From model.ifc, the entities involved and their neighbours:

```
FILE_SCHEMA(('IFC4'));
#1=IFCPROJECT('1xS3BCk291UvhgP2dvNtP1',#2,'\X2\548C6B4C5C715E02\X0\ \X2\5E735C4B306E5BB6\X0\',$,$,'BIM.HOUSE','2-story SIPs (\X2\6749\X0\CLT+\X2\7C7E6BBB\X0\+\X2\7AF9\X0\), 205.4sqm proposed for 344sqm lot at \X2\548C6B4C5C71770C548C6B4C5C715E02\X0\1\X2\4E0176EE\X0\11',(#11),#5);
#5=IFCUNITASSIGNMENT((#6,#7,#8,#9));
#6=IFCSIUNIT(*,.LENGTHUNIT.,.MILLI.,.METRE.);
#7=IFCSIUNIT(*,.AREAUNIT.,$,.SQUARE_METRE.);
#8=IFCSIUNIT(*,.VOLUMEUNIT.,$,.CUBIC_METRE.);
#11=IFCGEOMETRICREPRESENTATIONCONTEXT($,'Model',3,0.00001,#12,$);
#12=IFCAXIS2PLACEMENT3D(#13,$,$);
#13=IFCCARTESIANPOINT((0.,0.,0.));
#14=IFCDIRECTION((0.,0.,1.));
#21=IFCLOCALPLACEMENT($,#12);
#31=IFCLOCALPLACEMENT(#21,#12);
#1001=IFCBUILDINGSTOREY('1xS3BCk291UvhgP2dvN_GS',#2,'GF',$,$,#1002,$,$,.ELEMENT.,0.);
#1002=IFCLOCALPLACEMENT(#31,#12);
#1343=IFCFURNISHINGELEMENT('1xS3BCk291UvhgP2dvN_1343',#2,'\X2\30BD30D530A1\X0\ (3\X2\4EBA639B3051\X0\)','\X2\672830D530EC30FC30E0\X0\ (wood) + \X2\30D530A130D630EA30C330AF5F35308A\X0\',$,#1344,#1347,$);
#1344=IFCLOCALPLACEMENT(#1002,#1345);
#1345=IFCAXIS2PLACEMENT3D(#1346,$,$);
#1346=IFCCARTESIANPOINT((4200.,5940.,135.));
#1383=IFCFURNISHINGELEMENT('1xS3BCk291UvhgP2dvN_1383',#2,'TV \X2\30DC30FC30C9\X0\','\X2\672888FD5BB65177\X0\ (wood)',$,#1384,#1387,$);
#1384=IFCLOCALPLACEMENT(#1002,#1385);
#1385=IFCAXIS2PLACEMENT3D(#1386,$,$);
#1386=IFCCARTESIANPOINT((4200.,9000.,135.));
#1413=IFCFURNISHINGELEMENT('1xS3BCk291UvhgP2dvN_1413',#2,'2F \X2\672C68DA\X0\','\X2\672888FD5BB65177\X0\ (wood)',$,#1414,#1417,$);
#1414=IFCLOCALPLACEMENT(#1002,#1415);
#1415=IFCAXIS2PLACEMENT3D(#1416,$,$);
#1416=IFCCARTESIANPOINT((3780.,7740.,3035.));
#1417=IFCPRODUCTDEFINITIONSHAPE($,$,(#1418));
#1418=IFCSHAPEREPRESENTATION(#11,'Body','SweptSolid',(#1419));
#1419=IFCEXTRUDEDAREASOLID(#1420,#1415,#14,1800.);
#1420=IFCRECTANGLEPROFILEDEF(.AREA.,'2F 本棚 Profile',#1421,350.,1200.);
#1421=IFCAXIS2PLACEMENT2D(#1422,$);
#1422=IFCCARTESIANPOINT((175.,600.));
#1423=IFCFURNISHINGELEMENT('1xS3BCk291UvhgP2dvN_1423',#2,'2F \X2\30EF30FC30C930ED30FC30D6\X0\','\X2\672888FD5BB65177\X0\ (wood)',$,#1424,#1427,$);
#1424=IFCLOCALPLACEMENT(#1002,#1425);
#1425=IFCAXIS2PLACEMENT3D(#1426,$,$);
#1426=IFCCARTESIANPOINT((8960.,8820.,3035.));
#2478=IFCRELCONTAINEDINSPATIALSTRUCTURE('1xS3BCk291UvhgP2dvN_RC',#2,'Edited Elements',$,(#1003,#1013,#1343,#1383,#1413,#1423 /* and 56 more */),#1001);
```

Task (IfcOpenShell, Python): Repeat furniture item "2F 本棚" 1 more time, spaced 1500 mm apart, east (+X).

```python
import numpy as np
import ifcopenshell
import ifcopenshell.api.geometry
import ifcopenshell.api.root
import ifcopenshell.util.element
import ifcopenshell.util.placement

model = ifcopenshell.open("model.ifc")


def reuse_history(source, copy):
    """copy_class also copies each property set's owner history, people and application; keep the originals."""
    for rel in copy.IsDefinedBy:
        if rel.is_a("IfcRelDefinesByProperties") and (history := rel.RelatingPropertyDefinition.OwnerHistory):
            rel.RelatingPropertyDefinition.OwnerHistory = source.OwnerHistory
            ifcopenshell.util.element.remove_deep2(model, history)


source = model.by_guid("1xS3BCk291UvhgP2dvN_1413")
base = ifcopenshell.util.placement.get_local_placement(source.ObjectPlacement)
step = np.array([1.0, 0.0, 0.0]) * 1500.0

for i in range(1, 2):
    copy = ifcopenshell.api.root.copy_class(model, product=source)
    copy.Representation = ifcopenshell.util.element.copy_deep(
        model, source.Representation, exclude=["IfcGeometricRepresentationContext", "IfcRepresentationMap"]
    )
    reuse_history(source, copy)
    matrix = base.copy()
    matrix[:3, 3] += i * step
    print("added at", matrix[:3, 3].round(3) + 0.0)
    ifcopenshell.api.geometry.edit_object_placement(model, product=copy, matrix=matrix, is_si=False)

model.write("model-out.ifc")
```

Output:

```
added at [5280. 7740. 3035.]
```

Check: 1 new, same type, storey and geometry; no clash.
